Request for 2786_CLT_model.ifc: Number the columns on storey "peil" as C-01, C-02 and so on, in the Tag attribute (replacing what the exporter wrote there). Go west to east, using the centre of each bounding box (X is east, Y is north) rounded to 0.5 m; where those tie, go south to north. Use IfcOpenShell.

First a look at what the model holds.

```python
import ifcopenshell
import ifcopenshell.util.element
import ifcopenshell.util.placement

model = ifcopenshell.open("2786_CLT_model.ifc")
print(model.schema)
storey = next(s for s in model.by_type("IfcBuildingStorey") if s.Name == "peil")
columns = [e for e in ifcopenshell.util.element.get_decomposition(storey) if e.is_a("IfcColumn")]
for e in sorted(columns, key=lambda e: e.id()):
    origin = ifcopenshell.util.placement.get_local_placement(e.ObjectPlacement)[:3, 3]
    print(e.id(), e.Tag, e.Name, origin.round(2) + 0.0, sep=" | ")
```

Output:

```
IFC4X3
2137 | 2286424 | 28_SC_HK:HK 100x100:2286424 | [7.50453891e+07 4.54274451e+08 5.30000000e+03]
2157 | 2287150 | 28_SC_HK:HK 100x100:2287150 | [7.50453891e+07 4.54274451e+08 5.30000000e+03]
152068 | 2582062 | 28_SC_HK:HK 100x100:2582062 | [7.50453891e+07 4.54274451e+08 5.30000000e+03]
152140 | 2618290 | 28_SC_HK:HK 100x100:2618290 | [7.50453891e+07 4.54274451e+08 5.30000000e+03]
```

```python
import ifcopenshell
import ifcopenshell.geom
import ifcopenshell.util.element
import ifcopenshell.util.shape

model = ifcopenshell.open("2786_CLT_model.ifc")
settings = ifcopenshell.geom.settings()
settings.set("use-world-coords", True)


def centre(element):
    shape = ifcopenshell.geom.create_shape(settings, element)
    return ifcopenshell.util.shape.get_bbox_centroid(shape.geometry)


storey = next(s for s in model.by_type("IfcBuildingStorey") if s.Name == "peil")
columns = [e for e in ifcopenshell.util.element.get_decomposition(storey) if e.is_a("IfcColumn")]

# Insertion points can sit at a corner or the storey origin, so sort by the geometry (in metres).
centres = {e: centre(e) for e in columns}
columns.sort(key=lambda e: (round(centres[e][0] / 0.5), centres[e][1]))

for i, e in enumerate(columns, start=1):
    number = f"C-{i:02d}"
    e.Tag = number
    print(e.id(), number)

model.write("2786_CLT_model_rev.ifc")
```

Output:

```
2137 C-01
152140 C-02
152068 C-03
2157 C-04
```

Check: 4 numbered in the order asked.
